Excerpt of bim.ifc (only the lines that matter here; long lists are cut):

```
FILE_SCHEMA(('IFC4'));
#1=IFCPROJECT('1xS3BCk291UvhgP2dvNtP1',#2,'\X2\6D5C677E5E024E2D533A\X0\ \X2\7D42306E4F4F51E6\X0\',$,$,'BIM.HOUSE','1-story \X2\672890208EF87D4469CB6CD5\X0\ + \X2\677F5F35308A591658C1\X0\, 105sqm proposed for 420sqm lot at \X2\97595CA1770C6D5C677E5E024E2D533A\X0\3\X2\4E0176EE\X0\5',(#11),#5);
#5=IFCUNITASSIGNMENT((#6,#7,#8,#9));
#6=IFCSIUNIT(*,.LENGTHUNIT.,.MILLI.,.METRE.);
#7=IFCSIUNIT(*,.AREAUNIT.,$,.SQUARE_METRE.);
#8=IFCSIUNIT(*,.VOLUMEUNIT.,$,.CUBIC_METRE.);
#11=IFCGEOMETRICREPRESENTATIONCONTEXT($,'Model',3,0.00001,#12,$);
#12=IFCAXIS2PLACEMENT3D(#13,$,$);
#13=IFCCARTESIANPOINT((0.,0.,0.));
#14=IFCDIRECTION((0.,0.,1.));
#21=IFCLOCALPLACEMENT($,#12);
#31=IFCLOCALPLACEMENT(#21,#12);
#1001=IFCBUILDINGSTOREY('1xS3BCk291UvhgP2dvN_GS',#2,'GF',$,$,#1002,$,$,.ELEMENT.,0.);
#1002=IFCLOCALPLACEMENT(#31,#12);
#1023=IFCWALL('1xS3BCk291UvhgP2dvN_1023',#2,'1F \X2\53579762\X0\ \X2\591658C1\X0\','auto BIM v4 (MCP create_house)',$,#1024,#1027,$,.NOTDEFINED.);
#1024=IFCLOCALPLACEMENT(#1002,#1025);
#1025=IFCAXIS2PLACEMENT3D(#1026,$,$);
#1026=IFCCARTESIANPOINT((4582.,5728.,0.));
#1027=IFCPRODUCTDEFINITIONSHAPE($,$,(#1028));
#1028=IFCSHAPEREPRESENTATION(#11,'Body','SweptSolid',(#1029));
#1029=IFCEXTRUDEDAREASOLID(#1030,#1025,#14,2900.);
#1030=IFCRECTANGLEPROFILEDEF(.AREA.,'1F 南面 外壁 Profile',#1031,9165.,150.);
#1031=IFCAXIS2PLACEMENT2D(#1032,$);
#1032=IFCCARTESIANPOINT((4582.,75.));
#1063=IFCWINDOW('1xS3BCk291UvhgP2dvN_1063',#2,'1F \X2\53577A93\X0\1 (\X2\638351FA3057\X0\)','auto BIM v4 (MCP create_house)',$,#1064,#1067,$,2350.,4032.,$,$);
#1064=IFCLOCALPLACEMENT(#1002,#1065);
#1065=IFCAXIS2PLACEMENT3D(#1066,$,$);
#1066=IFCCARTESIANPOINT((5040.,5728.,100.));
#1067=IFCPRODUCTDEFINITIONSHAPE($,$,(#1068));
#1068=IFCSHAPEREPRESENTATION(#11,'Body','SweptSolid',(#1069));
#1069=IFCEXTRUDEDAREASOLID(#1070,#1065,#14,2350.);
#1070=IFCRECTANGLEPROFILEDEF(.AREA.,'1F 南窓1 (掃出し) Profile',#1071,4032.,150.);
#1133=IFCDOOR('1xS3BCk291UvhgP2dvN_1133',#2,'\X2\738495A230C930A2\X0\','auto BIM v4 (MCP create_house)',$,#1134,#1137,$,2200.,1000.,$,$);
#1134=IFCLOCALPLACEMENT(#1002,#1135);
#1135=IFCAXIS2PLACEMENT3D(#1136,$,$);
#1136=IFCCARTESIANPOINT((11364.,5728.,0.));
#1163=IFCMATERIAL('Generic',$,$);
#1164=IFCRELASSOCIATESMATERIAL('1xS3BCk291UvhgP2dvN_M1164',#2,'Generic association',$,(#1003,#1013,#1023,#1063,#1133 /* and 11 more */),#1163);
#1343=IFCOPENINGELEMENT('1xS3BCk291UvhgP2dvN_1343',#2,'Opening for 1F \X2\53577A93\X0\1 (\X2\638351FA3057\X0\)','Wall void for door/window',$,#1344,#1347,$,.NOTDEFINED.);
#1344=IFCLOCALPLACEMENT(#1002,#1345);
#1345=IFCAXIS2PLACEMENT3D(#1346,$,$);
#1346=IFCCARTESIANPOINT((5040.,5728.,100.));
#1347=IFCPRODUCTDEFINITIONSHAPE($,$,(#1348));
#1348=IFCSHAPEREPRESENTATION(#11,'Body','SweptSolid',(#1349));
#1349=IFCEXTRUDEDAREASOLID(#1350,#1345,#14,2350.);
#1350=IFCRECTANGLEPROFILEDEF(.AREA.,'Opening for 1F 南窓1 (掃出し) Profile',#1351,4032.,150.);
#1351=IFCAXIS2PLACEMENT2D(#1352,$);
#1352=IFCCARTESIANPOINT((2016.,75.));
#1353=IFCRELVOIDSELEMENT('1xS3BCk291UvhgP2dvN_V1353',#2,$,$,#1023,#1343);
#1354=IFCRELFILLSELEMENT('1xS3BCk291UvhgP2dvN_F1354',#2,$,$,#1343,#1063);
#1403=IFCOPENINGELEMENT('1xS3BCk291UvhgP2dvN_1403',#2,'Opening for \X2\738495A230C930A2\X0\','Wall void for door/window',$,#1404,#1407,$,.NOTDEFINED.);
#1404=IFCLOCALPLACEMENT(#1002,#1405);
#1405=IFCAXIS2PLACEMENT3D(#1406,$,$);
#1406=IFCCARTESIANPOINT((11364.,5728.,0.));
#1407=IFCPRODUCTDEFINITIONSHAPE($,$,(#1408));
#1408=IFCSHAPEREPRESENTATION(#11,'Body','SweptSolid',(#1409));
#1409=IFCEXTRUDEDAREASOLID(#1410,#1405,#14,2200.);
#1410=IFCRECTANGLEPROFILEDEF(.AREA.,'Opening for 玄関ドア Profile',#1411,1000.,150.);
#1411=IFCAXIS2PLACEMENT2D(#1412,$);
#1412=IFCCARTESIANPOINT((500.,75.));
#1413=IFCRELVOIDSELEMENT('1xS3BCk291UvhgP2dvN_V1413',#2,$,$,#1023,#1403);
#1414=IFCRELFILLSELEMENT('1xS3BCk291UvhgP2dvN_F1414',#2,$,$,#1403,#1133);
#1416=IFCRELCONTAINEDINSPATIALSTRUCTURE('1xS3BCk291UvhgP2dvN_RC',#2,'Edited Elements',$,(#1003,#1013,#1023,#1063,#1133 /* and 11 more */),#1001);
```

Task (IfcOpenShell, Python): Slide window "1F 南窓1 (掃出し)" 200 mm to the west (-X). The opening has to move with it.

```python
import ifcopenshell
import ifcopenshell.api.geometry
import ifcopenshell.util.placement
import ifcopenshell.util.unit

model = ifcopenshell.open("bim.ifc")
unit_scale = ifcopenshell.util.unit.calculate_unit_scale(model)

window = model.by_guid("1xS3BCk291UvhgP2dvN_1063")
opening = window.FillsVoids[0].RelatingOpeningElement
wall = opening.VoidsElements[0].RelatingBuildingElement

wall_matrix = ifcopenshell.util.placement.get_local_placement(wall.ObjectPlacement)
shift = wall_matrix[:3, 0] * -0.2 / unit_scale
before = ifcopenshell.util.placement.get_local_placement(window.ObjectPlacement)[:3, 3].copy()

# The window is not placed relative to its opening, so move both.
for product in (opening, window):
    matrix = ifcopenshell.util.placement.get_local_placement(product.ObjectPlacement)
    matrix[:3, 3] += shift
    ifcopenshell.api.geometry.edit_object_placement(model, product=product, matrix=matrix, is_si=False)

after = ifcopenshell.util.placement.get_local_placement(window.ObjectPlacement)[:3, 3]
print("window moved by", (after - before).round(3) + 0.0)

model.write("bim_updated.ifc")
```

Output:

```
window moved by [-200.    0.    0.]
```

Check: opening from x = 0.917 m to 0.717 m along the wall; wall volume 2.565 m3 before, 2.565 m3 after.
